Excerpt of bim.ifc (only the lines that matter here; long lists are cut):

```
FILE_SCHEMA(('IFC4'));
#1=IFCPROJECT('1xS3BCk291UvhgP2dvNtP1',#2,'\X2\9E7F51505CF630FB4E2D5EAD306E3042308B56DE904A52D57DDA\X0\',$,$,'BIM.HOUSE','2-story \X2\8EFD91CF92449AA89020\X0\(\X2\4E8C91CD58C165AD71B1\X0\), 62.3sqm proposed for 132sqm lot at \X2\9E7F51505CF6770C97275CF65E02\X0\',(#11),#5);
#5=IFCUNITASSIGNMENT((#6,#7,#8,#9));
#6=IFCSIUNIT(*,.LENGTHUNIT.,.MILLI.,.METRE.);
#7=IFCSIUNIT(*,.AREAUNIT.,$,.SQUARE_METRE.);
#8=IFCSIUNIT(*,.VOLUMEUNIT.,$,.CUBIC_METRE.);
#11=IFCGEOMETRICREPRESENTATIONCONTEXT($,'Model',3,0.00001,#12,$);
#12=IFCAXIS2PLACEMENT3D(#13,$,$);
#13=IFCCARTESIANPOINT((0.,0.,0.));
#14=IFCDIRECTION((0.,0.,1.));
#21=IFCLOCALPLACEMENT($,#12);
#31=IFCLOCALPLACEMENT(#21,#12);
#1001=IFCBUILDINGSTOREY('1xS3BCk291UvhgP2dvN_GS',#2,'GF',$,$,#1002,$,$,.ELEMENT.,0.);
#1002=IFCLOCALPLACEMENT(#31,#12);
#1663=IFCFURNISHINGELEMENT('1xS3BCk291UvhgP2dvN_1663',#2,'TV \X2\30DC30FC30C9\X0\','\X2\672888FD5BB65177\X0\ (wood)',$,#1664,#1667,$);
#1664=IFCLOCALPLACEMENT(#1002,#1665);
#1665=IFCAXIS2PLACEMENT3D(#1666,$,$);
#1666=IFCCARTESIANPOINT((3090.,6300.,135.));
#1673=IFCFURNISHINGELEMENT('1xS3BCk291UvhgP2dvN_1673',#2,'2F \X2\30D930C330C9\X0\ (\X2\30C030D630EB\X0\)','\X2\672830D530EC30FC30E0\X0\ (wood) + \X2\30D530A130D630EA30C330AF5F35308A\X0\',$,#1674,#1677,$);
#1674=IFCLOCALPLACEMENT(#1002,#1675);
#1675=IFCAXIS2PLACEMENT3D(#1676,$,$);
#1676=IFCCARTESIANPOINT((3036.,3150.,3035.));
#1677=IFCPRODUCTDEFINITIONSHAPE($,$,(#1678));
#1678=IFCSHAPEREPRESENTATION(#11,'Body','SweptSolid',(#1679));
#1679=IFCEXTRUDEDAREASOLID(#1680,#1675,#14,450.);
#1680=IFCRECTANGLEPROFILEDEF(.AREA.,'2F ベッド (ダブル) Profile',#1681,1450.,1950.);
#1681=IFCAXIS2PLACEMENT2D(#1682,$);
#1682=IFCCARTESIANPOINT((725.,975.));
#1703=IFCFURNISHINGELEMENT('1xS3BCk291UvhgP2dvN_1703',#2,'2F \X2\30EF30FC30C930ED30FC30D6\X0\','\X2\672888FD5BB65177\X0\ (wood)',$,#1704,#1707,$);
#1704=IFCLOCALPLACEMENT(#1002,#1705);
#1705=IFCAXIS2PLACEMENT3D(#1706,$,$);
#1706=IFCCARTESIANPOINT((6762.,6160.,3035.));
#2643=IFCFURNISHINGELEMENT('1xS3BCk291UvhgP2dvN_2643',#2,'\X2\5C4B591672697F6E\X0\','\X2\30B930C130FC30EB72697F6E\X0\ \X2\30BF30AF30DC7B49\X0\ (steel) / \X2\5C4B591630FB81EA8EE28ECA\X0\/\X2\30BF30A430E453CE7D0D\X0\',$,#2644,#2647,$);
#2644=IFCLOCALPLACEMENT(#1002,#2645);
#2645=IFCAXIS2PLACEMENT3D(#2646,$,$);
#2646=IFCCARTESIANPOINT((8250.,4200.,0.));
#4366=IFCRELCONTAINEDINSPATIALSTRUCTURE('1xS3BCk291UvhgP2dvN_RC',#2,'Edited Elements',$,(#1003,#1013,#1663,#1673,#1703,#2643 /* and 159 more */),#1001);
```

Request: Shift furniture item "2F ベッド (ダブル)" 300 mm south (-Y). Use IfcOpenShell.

```python
import ifcopenshell
import ifcopenshell.api.geometry
import ifcopenshell.util.placement
import ifcopenshell.util.unit

model = ifcopenshell.open("bim.ifc")
unit_scale = ifcopenshell.util.unit.calculate_unit_scale(model)

item = model.by_guid("1xS3BCk291UvhgP2dvN_1673")
matrix = ifcopenshell.util.placement.get_local_placement(item.ObjectPlacement)
matrix[1, 3] -= 0.3 / unit_scale
ifcopenshell.api.geometry.edit_object_placement(model, product=item, matrix=matrix, is_si=False)

print(ifcopenshell.util.placement.get_local_placement(item.ObjectPlacement).round(3) + 0.0)

model.write("bim_updated.ifc")
```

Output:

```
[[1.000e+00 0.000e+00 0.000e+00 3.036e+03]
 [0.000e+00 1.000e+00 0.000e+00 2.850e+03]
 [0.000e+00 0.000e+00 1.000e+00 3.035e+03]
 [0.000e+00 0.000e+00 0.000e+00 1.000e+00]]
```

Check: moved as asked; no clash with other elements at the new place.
